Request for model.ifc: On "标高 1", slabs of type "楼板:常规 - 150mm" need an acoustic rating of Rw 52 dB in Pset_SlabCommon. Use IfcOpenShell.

First a look at what the model holds.

```python
import ifcopenshell
import ifcopenshell.util.element

model = ifcopenshell.open("model.ifc")
print(model.schema)
storey = next(s for s in model.by_type("IfcBuildingStorey") if s.Name == "标高 1")
slabs = [e for e in ifcopenshell.util.element.get_decomposition(storey) if e.is_a("IfcSlab")]
seen = {}
for e in slabs:
    element_type = ifcopenshell.util.element.get_type(e)
    key = (element_type.Name if element_type != e and element_type else None, ifcopenshell.util.element.get_pset(e, "Pset_SlabCommon", "AcousticRating"))
    seen[key] = seen.get(key, 0) + 1
for (name, value), count in sorted(seen.items(), key=str):
    print(count, "x", name, "|", value)
```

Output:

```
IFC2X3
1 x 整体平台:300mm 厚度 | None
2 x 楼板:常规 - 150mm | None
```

```python
import ifcopenshell
import ifcopenshell.api.pset
import ifcopenshell.util.element

model = ifcopenshell.open("model.ifc")

storey = next(s for s in model.by_type("IfcBuildingStorey") if s.Name == "标高 1")
slabs = [e for e in ifcopenshell.util.element.get_decomposition(storey) if e.is_a("IfcSlab")]

count = 0
for e in slabs:
    element_type = ifcopenshell.util.element.get_type(e)
    if element_type in (None, e) or element_type.Name != "楼板:常规 - 150mm":
        continue
    # add_pset returns the element's existing set when there is one.
    pset = ifcopenshell.api.pset.add_pset(model, product=e, name="Pset_SlabCommon")
    ifcopenshell.api.pset.edit_pset(model, pset=pset, properties={"AcousticRating": "Rw 52 dB"})
    count += 1

print(count, "slabs updated")

model.write("model-out.ifc")
```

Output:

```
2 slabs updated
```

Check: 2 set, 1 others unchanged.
